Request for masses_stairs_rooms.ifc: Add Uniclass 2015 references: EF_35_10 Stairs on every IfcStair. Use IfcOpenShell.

First a look at what the model holds.

```python
import ifcopenshell

model = ifcopenshell.open("masses_stairs_rooms.ifc")
print(model.schema)
print("classifications:", [c.Name for c in model.by_type("IfcClassification")])
for ifc_class in ("IfcDoor", "IfcRoof", "IfcStair", "IfcWall", "IfcWindow"):
    print(ifc_class, len(model.by_type(ifc_class)))
```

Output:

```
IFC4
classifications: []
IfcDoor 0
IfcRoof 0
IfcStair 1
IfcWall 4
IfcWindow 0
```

```python
import ifcopenshell
import ifcopenshell.api.classification

model = ifcopenshell.open("masses_stairs_rooms.ifc")

system = ifcopenshell.api.classification.add_classification(model, classification="Uniclass 2015")

codes = {
    "IfcStair": ("EF_35_10", "Stairs"),
}
for ifc_class, (code, name) in codes.items():
    products = model.by_type(ifc_class)
    ifcopenshell.api.classification.add_reference(
        model, products=products, classification=system, identification=code, name=name
    )
    print(code, len(products))

model.write("masses_stairs_rooms_rev.ifc")
```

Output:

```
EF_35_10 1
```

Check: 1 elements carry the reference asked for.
